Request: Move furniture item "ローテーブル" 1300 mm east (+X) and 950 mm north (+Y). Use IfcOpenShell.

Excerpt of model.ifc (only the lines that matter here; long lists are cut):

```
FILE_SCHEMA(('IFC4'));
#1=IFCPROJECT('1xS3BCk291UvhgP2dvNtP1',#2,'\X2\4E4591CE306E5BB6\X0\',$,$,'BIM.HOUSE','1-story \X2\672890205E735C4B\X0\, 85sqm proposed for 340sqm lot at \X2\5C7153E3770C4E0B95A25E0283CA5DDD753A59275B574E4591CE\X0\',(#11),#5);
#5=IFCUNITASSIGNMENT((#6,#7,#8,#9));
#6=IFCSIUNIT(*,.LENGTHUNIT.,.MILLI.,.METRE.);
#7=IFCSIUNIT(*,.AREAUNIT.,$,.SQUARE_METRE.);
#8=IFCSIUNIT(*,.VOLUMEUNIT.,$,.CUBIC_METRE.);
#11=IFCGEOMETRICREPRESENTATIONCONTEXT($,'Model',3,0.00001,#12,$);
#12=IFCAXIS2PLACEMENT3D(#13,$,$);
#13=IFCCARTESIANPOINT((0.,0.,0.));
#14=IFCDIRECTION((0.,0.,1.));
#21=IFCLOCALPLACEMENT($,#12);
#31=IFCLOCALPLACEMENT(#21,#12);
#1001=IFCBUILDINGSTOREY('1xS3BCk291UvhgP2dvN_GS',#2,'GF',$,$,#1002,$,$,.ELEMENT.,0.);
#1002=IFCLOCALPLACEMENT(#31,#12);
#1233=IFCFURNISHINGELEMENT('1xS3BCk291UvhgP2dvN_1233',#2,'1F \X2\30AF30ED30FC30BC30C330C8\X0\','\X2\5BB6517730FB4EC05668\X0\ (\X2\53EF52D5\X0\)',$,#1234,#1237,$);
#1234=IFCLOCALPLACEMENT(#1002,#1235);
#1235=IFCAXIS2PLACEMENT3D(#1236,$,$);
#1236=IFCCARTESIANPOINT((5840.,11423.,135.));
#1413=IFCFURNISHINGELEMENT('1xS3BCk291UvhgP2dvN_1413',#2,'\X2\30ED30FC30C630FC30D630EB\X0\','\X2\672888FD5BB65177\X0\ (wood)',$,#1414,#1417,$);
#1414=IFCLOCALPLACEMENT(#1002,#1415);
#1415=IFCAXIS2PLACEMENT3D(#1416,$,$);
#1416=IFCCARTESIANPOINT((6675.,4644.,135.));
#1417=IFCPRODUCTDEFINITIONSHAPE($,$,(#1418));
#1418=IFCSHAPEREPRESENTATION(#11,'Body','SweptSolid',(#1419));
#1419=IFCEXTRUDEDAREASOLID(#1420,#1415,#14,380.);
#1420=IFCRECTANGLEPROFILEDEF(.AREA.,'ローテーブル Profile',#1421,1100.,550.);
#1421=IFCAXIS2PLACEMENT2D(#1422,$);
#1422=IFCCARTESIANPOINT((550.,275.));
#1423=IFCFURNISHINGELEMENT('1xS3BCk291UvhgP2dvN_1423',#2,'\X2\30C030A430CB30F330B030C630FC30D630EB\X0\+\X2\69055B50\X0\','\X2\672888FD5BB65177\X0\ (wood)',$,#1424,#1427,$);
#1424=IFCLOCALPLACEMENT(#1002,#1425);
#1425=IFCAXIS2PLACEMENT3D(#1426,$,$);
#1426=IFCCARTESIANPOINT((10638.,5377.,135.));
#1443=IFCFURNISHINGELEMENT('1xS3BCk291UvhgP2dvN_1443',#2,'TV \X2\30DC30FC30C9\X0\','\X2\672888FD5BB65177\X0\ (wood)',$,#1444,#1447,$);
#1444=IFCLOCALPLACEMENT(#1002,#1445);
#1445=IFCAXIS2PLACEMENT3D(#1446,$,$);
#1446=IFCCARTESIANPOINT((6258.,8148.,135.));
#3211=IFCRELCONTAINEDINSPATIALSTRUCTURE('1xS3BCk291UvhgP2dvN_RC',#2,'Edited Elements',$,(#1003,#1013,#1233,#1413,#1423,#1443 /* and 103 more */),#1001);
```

```python
import ifcopenshell
import ifcopenshell.api.geometry
import ifcopenshell.util.placement
import ifcopenshell.util.unit

model = ifcopenshell.open("model.ifc")
unit_scale = ifcopenshell.util.unit.calculate_unit_scale(model)

item = model.by_guid("1xS3BCk291UvhgP2dvN_1413")
matrix = ifcopenshell.util.placement.get_local_placement(item.ObjectPlacement)
matrix[0, 3] += 1.3 / unit_scale
matrix[1, 3] += 0.95 / unit_scale
ifcopenshell.api.geometry.edit_object_placement(model, product=item, matrix=matrix, is_si=False)

print(ifcopenshell.util.placement.get_local_placement(item.ObjectPlacement).round(3) + 0.0)

model.write("model-out.ifc")
```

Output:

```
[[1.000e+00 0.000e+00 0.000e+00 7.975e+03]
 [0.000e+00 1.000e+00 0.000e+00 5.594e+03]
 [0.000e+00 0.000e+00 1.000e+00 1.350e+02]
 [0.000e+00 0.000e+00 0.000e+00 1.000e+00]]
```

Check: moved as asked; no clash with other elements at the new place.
